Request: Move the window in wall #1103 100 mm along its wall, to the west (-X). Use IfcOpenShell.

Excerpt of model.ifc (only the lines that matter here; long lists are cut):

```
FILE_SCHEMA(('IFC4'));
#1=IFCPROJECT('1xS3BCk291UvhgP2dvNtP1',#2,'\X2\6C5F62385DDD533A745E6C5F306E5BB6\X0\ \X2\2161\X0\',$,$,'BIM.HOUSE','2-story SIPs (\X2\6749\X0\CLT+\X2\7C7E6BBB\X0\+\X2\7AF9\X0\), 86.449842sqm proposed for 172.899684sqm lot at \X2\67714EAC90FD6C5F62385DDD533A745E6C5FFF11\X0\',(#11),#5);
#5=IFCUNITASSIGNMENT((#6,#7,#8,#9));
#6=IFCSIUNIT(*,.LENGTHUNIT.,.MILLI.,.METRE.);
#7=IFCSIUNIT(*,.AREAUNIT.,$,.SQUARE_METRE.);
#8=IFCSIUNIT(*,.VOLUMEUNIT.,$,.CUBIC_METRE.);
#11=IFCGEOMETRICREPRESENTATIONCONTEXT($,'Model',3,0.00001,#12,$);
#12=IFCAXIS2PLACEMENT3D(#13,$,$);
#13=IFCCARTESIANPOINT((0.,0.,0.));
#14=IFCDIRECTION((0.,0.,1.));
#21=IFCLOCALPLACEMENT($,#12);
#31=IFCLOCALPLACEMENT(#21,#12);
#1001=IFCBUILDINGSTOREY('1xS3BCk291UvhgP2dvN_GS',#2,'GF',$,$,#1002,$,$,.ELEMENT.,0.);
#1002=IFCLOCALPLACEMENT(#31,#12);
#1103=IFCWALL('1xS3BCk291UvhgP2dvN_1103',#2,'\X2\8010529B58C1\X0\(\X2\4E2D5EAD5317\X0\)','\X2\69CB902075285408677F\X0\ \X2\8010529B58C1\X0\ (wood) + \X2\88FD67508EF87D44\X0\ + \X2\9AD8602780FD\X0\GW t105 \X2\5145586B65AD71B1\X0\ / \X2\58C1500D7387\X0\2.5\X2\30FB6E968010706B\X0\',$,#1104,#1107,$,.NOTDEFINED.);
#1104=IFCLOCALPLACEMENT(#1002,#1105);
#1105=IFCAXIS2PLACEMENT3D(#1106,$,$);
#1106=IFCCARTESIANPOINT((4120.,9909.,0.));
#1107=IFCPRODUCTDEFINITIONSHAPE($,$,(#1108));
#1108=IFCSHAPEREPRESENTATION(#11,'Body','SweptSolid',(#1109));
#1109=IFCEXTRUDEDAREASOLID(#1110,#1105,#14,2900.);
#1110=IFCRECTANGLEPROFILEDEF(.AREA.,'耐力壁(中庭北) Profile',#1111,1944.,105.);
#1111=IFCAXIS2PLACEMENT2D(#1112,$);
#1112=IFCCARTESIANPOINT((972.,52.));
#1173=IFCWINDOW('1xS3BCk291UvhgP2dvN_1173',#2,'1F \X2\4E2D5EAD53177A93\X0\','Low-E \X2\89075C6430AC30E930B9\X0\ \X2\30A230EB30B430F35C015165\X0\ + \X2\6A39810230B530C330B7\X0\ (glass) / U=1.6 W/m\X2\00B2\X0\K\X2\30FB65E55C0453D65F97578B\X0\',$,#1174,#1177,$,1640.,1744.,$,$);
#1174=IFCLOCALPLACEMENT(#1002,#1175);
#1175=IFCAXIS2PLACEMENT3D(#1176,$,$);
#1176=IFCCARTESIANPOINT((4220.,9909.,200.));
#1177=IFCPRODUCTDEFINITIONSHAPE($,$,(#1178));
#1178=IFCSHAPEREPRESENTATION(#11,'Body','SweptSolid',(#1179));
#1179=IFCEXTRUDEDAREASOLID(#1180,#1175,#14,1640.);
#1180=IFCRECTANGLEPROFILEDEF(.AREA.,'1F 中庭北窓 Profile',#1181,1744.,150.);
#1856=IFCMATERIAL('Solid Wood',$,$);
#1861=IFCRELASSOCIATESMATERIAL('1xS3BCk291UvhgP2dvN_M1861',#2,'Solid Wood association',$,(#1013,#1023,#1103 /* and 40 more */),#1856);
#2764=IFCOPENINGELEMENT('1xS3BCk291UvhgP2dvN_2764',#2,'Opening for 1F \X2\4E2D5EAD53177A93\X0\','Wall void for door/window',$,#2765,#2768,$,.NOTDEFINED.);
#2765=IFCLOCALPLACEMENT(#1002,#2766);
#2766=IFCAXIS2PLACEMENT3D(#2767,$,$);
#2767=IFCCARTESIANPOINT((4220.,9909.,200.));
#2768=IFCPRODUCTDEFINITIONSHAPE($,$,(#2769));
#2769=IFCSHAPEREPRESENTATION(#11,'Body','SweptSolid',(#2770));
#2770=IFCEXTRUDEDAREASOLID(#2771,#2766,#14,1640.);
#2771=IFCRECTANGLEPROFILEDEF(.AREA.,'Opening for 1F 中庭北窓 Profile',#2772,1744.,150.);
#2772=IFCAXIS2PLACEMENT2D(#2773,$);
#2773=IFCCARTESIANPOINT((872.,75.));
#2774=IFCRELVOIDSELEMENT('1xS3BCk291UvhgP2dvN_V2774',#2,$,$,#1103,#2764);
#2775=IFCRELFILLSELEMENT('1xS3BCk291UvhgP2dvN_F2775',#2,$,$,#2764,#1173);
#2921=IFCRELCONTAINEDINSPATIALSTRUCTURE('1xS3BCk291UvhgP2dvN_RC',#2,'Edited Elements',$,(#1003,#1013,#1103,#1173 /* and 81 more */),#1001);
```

```python
import ifcopenshell
import ifcopenshell.api.geometry
import ifcopenshell.util.placement

model = ifcopenshell.open("model.ifc")

window = model.by_id(1173)
opening = window.FillsVoids[0].RelatingOpeningElement
wall = opening.VoidsElements[0].RelatingBuildingElement

wall_matrix = ifcopenshell.util.placement.get_local_placement(wall.ObjectPlacement)
shift = wall_matrix[:3, 0] * -100.0
before = ifcopenshell.util.placement.get_local_placement(window.ObjectPlacement)[:3, 3].copy()

# The window is not placed relative to its opening, so move both.
for product in (opening, window):
    matrix = ifcopenshell.util.placement.get_local_placement(product.ObjectPlacement)
    matrix[:3, 3] += shift
    ifcopenshell.api.geometry.edit_object_placement(model, product=product, matrix=matrix, is_si=False)

after = ifcopenshell.util.placement.get_local_placement(window.ObjectPlacement)[:3, 3]
print("window moved by", (after - before).round(3) + 0.0)

model.write("model_updated.ifc")
```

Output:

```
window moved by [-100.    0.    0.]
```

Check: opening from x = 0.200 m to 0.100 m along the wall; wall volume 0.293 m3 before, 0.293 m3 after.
